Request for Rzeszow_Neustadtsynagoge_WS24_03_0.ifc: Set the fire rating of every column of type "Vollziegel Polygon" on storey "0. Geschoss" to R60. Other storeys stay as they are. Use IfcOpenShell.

First a look at what the model holds.

```python
import ifcopenshell
import ifcopenshell.util.element

model = ifcopenshell.open("Rzeszow_Neustadtsynagoge_WS24_03_0.ifc")
print(model.schema)
storey = next(s for s in model.by_type("IfcBuildingStorey") if s.Name == "0. Geschoss")
columns = [e for e in ifcopenshell.util.element.get_decomposition(storey) if e.is_a("IfcColumn")]
seen = {}
for e in columns:
    element_type = ifcopenshell.util.element.get_type(e)
    key = (element_type.Name if element_type != e and element_type else None, ifcopenshell.util.element.get_pset(e, "Pset_ColumnCommon", "FireRating"))
    seen[key] = seen.get(key, 0) + 1
for (name, value), count in sorted(seen.items(), key=str):
    print(count, "x", name, "|", value)
```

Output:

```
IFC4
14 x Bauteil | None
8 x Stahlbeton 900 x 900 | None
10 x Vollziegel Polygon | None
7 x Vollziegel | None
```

```python
import ifcopenshell
import ifcopenshell.api.pset
import ifcopenshell.util.element

model = ifcopenshell.open("Rzeszow_Neustadtsynagoge_WS24_03_0.ifc")

storey = next(s for s in model.by_type("IfcBuildingStorey") if s.Name == "0. Geschoss")
columns = [e for e in ifcopenshell.util.element.get_decomposition(storey) if e.is_a("IfcColumn")]

count = 0
for e in columns:
    element_type = ifcopenshell.util.element.get_type(e)
    if element_type in (None, e) or element_type.Name != "Vollziegel Polygon":
        continue
    # add_pset returns the element's existing set when there is one.
    pset = ifcopenshell.api.pset.add_pset(model, product=e, name="Pset_ColumnCommon")
    ifcopenshell.api.pset.edit_pset(model, pset=pset, properties={"FireRating": "R60"})
    count += 1

print(count, "columns updated")

model.write("Rzeszow_Neustadtsynagoge_WS24_03_0_edited.ifc")
```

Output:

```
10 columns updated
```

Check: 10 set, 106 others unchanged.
